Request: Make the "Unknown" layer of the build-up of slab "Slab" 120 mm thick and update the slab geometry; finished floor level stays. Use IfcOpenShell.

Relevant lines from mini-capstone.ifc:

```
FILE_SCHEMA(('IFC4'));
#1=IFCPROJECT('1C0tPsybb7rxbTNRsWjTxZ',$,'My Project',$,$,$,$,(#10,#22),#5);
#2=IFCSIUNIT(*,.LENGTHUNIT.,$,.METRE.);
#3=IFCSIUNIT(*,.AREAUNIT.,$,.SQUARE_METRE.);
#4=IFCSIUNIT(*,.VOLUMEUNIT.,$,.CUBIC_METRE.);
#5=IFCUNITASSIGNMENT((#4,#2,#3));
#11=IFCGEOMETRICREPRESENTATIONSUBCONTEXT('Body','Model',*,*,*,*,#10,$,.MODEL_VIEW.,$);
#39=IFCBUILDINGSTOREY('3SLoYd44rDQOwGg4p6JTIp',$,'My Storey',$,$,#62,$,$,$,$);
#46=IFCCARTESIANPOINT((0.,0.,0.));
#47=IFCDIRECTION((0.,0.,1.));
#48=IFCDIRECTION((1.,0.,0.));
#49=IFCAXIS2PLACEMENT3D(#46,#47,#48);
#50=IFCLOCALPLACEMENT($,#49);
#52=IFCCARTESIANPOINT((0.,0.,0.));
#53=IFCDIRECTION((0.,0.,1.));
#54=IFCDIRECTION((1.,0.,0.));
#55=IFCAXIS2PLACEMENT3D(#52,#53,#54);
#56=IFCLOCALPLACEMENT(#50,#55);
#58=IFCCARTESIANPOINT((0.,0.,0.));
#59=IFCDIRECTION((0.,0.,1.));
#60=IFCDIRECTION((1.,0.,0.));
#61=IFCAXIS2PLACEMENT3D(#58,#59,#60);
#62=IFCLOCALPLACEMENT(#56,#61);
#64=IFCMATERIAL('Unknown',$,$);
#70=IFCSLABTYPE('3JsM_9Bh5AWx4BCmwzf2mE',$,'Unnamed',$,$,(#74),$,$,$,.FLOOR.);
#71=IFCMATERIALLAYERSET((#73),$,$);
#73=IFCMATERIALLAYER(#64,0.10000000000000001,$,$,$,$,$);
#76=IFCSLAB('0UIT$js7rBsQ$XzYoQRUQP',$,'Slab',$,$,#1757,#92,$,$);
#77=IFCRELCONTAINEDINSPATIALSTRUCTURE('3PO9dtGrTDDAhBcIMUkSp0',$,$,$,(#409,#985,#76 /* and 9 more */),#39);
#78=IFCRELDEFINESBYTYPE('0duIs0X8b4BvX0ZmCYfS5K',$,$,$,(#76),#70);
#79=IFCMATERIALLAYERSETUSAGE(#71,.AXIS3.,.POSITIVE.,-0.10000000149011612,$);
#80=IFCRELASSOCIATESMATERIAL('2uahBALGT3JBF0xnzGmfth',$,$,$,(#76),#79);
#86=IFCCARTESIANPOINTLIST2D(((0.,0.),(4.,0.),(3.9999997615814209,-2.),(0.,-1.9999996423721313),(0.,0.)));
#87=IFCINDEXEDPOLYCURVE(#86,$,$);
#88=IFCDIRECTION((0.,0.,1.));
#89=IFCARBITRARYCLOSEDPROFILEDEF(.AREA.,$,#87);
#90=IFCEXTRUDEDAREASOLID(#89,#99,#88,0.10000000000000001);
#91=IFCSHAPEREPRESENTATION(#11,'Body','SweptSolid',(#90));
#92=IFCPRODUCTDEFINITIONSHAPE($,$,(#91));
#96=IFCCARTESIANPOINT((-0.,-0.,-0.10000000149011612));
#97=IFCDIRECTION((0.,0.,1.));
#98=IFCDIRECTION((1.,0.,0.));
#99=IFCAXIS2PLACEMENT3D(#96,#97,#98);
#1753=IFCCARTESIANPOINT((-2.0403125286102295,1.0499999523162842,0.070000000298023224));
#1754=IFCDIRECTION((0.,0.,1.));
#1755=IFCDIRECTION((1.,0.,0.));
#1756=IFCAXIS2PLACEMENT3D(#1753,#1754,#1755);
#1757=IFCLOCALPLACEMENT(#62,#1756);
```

```python
import ifcopenshell
import ifcopenshell.util.element
import ifcopenshell.util.representation

model = ifcopenshell.open("mini-capstone.ifc")

layer_set = model.by_id(71)
layer = next(l for l in layer_set.MaterialLayers if l.Material and l.Material.Name == "Unknown")
change = 0.12 - layer.LayerThickness
layer.LayerThickness += change

# Geometry does not follow the layer set by itself.
slabs = [e for e in ifcopenshell.util.element.get_elements_by_material(model, layer_set) if e.is_a("IfcSlab")]
for slab in sorted(slabs, key=lambda e: e.id()):
    body = ifcopenshell.util.representation.get_representation(slab, "Model", "Body")
    solid = body.Items[0]
    old_depth = solid.Depth
    solid.Depth += change
    # Extruded upwards: lower the start of the extrusion so the top stays.
    x, y, z = solid.Position.Location.Coordinates
    solid.Position.Location = model.createIfcCartesianPoint((x, y, z - change))
    print(slab.id(), f"{old_depth:g} -> {solid.Depth:g}")

# The layers are counted up from the underside, which has moved.
for usage in {ifcopenshell.util.element.get_material(slab) for slab in slabs}:
    usage.OffsetFromReferenceLine -= change

model.write("mini-capstone_edited.ifc")
```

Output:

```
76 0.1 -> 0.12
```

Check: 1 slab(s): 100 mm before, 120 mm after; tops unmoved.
